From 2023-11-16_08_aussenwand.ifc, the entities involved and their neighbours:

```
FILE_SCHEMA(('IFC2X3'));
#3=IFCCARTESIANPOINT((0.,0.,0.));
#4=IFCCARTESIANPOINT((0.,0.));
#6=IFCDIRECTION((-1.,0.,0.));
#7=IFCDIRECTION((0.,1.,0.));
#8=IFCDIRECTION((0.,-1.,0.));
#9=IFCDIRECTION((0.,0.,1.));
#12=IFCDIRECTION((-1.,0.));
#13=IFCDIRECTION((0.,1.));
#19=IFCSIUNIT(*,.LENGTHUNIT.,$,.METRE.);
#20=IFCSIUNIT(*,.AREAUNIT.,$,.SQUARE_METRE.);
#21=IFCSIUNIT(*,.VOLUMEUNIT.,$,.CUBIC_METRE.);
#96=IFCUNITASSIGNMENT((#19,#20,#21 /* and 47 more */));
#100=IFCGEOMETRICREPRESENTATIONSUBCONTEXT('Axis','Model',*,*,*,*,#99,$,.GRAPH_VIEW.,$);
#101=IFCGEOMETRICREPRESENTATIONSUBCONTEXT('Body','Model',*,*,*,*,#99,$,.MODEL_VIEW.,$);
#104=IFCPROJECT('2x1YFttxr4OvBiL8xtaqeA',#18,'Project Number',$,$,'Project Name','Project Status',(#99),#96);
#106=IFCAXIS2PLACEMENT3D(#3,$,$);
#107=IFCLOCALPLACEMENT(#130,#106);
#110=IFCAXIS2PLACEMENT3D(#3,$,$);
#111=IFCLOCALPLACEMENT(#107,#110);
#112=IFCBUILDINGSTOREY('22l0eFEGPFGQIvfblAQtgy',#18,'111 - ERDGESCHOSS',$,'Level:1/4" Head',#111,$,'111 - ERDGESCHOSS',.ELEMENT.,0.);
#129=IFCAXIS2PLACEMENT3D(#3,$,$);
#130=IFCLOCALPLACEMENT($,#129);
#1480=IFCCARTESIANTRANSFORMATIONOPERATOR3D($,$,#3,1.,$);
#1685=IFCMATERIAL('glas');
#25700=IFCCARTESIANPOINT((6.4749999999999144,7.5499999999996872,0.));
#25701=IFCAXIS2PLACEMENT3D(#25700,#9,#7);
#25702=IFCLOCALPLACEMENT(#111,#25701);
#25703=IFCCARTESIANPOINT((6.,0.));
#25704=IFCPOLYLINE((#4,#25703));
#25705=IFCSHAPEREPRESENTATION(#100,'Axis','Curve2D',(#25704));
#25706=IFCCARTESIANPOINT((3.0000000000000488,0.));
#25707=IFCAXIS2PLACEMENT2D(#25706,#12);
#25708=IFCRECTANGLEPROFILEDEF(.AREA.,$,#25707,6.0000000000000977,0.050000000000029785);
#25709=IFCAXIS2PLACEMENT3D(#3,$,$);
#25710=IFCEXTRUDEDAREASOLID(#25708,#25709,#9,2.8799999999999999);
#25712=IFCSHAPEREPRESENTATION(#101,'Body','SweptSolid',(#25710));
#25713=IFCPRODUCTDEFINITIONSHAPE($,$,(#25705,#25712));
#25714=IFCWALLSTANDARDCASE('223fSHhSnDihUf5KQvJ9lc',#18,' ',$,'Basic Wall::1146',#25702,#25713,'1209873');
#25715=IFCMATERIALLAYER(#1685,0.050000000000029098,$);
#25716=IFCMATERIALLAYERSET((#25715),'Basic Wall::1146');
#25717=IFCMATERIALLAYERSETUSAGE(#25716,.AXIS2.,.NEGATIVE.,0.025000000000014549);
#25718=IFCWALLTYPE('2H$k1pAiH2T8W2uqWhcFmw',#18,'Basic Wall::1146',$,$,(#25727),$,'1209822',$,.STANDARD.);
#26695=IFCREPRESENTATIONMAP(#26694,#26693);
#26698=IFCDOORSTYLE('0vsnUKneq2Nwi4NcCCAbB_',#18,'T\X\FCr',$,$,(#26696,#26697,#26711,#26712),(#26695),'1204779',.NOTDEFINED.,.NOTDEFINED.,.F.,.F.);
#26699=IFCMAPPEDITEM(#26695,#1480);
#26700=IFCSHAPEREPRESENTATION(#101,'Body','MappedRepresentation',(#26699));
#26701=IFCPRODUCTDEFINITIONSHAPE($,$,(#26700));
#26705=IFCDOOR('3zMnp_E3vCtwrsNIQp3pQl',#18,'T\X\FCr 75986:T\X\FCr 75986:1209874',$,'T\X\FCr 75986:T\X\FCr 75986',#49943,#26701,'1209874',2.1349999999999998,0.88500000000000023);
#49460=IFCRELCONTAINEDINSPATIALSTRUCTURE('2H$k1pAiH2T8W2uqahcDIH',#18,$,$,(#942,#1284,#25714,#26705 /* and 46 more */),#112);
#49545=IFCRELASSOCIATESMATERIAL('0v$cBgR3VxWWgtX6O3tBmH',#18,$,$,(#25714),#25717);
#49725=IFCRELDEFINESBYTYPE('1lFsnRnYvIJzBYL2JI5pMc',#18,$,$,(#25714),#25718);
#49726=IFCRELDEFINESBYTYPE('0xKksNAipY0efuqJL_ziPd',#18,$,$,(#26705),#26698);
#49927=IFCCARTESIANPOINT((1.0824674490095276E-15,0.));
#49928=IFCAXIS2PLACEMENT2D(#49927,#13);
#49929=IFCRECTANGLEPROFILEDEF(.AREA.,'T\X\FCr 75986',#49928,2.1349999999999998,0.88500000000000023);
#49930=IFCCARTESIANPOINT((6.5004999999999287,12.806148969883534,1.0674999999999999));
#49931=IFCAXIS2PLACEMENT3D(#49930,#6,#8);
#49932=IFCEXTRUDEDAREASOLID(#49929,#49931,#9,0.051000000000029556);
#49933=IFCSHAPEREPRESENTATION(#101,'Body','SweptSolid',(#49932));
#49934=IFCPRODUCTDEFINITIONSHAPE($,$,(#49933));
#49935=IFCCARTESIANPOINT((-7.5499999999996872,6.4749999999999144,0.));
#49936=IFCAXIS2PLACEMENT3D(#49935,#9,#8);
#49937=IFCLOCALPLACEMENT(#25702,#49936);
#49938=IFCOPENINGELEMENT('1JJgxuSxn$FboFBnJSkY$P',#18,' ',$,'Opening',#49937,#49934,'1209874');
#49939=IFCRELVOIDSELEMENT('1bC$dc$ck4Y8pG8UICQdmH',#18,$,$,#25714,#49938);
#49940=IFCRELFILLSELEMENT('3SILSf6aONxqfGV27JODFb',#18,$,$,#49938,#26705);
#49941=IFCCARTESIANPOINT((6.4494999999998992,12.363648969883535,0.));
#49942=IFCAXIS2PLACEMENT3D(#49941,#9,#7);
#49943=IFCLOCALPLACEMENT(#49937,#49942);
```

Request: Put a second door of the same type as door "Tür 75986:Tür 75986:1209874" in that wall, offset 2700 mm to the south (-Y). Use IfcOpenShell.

```python
import ifcopenshell
import ifcopenshell.api.feature
import ifcopenshell.api.geometry
import ifcopenshell.api.root
import ifcopenshell.geom
import ifcopenshell.util.element
import ifcopenshell.util.placement
import ifcopenshell.util.shape
import ifcopenshell.util.unit

model = ifcopenshell.open("2023-11-16_08_aussenwand.ifc")
unit_scale = ifcopenshell.util.unit.calculate_unit_scale(model)
settings = ifcopenshell.geom.settings()


def volume(element):
    """Net volume in cubic metres, openings subtracted."""
    shape = ifcopenshell.geom.create_shape(settings, element)
    return ifcopenshell.util.shape.get_volume(shape.geometry)


def reuse_history(source, copy):
    """copy_class also copies each property set's owner history, people and application; keep the originals."""
    for rel in copy.IsDefinedBy:
        if rel.is_a("IfcRelDefinesByProperties") and (history := rel.RelatingPropertyDefinition.OwnerHistory):
            rel.RelatingPropertyDefinition.OwnerHistory = source.OwnerHistory
            ifcopenshell.util.element.remove_deep2(model, history)


door = model.by_guid("3zMnp_E3vCtwrsNIQp3pQl")
opening = door.FillsVoids[0].RelatingOpeningElement
wall = opening.VoidsElements[0].RelatingBuildingElement
before = volume(wall)
shift = ifcopenshell.util.placement.get_local_placement(wall.ObjectPlacement)[:3, 0] * -2.7 / unit_scale

# copy_class copies the void relationship, type, container and properties, but no geometry.
new_opening = ifcopenshell.api.root.copy_class(model, product=opening)
new_opening.Representation = ifcopenshell.util.element.copy_deep(
    model, opening.Representation, exclude=["IfcGeometricRepresentationContext", "IfcRepresentationMap"]
)
new_opening.Tag = None
new_door = ifcopenshell.api.root.copy_class(model, product=door)
new_door.Representation = ifcopenshell.util.element.copy_deep(
    model, door.Representation, exclude=["IfcGeometricRepresentationContext", "IfcRepresentationMap"]
)
new_door.Name = "Tür 75986:Tür 75986"
new_door.Tag = None
reuse_history(door, new_door)
fills = ifcopenshell.api.feature.add_filling(model, opening=new_opening, element=new_door)
fills.OwnerHistory = new_door.OwnerHistory  # required in IFC2X3

for old, new in ((opening, new_opening), (door, new_door)):
    matrix = ifcopenshell.util.placement.get_local_placement(old.ObjectPlacement)
    matrix[:3, 3] += shift
    ifcopenshell.api.geometry.edit_object_placement(model, product=new, matrix=matrix, is_si=False)

after = volume(wall)

print(f"wall volume {before:.3f} -> {after:.3f} m3")

model.write("2023-11-16_08_aussenwand_updated.ifc")
```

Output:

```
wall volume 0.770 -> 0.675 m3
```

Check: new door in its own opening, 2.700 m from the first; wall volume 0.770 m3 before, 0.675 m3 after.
